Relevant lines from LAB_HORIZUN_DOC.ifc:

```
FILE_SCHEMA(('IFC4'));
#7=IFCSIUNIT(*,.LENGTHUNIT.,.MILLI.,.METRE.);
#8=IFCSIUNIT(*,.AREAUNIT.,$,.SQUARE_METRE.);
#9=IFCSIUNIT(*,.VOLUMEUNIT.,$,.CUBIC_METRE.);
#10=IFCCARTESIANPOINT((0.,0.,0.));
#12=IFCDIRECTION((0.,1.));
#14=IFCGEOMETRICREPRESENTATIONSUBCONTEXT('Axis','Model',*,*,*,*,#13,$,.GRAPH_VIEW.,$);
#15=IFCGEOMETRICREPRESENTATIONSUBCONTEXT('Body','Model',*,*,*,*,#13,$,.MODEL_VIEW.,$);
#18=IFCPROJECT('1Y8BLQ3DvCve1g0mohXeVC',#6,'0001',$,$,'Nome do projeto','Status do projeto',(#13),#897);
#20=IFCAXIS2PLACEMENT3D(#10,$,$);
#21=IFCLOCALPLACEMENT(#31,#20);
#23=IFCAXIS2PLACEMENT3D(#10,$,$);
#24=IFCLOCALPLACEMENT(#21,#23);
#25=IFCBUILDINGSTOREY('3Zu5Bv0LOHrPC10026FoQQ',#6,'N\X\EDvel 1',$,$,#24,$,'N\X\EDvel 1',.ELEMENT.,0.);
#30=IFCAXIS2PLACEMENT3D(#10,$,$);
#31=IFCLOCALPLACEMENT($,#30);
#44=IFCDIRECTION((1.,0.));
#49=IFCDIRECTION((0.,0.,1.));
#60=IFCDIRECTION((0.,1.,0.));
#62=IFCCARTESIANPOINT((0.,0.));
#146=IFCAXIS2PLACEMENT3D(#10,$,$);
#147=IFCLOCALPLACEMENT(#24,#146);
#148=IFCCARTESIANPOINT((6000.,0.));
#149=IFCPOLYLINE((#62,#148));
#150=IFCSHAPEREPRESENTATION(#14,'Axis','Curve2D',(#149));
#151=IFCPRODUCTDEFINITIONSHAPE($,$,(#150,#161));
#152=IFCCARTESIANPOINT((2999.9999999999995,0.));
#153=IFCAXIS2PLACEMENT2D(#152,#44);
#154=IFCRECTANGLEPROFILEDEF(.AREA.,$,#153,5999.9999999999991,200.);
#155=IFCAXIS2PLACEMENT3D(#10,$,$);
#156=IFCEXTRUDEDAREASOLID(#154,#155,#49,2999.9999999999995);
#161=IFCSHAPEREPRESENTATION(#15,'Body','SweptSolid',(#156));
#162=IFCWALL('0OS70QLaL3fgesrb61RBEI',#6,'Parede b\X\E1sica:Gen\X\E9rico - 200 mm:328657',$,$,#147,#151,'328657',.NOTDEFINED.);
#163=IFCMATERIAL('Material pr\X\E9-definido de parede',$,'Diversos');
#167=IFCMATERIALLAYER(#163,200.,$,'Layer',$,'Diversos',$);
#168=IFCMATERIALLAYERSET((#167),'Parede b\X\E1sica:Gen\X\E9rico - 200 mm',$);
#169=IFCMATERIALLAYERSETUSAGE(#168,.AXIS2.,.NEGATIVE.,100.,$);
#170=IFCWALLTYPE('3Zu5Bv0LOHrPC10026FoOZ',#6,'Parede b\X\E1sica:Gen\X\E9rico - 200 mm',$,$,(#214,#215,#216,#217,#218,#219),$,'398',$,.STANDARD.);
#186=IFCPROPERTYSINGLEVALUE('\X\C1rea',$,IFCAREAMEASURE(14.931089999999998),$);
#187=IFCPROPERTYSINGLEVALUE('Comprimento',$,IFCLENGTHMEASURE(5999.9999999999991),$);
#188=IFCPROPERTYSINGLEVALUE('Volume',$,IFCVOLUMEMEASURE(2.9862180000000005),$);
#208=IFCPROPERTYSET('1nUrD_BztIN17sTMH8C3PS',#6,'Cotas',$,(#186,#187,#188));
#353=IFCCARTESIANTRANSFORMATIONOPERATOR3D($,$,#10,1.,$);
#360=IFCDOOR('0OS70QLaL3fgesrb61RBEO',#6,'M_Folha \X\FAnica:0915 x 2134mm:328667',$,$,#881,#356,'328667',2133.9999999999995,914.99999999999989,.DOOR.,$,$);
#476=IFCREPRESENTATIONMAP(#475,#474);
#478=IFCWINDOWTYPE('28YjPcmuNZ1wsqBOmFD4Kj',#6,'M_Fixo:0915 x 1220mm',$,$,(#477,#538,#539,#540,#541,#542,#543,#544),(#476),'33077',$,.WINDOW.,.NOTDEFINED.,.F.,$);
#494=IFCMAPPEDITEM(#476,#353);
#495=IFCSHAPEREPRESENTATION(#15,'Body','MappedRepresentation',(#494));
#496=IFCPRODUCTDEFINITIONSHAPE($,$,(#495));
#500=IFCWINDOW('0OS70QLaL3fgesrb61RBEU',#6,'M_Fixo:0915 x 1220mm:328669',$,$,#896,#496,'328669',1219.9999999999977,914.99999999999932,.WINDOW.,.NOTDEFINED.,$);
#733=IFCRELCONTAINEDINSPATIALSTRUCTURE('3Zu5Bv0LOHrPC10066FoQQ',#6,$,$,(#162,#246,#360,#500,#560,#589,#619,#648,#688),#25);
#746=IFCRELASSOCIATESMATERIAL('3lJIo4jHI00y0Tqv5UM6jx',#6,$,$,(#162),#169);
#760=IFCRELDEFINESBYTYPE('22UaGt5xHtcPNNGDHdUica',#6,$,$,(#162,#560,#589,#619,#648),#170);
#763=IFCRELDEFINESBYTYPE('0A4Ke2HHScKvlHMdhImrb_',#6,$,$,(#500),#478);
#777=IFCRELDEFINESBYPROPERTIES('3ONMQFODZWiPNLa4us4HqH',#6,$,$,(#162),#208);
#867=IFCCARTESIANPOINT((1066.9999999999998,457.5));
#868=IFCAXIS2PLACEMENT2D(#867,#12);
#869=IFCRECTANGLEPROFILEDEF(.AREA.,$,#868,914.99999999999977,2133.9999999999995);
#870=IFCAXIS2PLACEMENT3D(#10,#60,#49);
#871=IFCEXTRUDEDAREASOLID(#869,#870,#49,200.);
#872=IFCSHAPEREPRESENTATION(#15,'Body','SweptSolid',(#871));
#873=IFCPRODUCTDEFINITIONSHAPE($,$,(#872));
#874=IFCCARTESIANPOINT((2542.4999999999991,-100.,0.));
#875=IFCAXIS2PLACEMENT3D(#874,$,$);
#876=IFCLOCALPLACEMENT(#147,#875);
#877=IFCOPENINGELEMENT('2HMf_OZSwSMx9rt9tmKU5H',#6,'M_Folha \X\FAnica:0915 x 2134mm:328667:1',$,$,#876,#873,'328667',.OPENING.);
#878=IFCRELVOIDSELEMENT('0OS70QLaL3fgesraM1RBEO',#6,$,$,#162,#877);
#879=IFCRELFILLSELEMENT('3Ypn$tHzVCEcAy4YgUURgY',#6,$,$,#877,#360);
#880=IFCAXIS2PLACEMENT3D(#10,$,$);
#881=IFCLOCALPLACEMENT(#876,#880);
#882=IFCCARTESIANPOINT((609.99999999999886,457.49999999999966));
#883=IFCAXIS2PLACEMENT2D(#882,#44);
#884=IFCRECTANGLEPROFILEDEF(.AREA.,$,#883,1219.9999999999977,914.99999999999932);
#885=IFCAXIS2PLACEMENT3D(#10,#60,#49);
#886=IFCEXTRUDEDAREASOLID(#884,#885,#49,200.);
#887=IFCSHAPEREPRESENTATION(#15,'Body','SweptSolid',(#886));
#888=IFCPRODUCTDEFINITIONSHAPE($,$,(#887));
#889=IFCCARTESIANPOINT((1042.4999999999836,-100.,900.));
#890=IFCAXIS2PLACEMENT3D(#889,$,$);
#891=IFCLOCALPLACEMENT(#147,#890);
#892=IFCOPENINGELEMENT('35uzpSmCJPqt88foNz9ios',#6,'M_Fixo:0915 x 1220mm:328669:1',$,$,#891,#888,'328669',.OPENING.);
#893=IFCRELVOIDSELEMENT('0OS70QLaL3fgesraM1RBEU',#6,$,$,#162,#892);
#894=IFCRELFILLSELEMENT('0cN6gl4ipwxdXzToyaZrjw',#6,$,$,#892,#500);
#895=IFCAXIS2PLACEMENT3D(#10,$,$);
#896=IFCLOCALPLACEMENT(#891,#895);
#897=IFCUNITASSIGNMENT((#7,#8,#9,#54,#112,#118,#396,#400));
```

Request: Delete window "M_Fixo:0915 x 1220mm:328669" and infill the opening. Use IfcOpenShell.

```python
import ifcopenshell
import ifcopenshell.api.feature
import ifcopenshell.api.pset
import ifcopenshell.api.root
import ifcopenshell.geom
import ifcopenshell.util.element
import ifcopenshell.util.shape
import ifcopenshell.util.unit

model = ifcopenshell.open("LAB_HORIZUN_DOC.ifc")
area_scale = ifcopenshell.util.unit.calculate_unit_scale(model, "AREAUNIT")
volume_scale = ifcopenshell.util.unit.calculate_unit_scale(model, "VOLUMEUNIT")
settings = ifcopenshell.geom.settings()


def volume(element):
    """Net volume in cubic metres, openings subtracted."""
    shape = ifcopenshell.geom.create_shape(settings, element)
    return ifcopenshell.util.shape.get_volume(shape.geometry)


window = model.by_id(500)
opening = window.FillsVoids[0].RelatingOpeningElement
wall = opening.VoidsElements[0].RelatingBuildingElement
before = volume(wall)

ifcopenshell.api.root.remove_product(model, product=window)
ifcopenshell.api.feature.remove_feature(model, feature=opening)

after = volume(wall)
thickness = 0.2  # wall thickness in metres

# Update the wall's stored quantities.
pset = model.by_id(ifcopenshell.util.element.get_pset(wall, "Cotas", should_inherit=False)["id"])
ifcopenshell.api.pset.edit_pset(model, pset=pset, properties={
    "Área": model.create_entity("IfcAreaMeasure", after / thickness / area_scale),
    "Volume": model.create_entity("IfcVolumeMeasure", after / volume_scale),
})

print(f"wall volume {before:.3f} -> {after:.3f} m3")

model.write("LAB_HORIZUN_DOC_edited.ifc")
```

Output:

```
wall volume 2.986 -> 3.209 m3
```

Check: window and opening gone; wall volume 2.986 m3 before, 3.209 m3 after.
